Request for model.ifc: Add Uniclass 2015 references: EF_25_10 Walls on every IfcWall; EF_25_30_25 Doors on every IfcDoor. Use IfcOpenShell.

First a look at what the model holds.

```python
import ifcopenshell

model = ifcopenshell.open("model.ifc")
print(model.schema)
print("classifications:", [c.Name for c in model.by_type("IfcClassification")])
for ifc_class in ("IfcDoor", "IfcRoof", "IfcStair", "IfcWall", "IfcWindow"):
    print(ifc_class, len(model.by_type(ifc_class)))
```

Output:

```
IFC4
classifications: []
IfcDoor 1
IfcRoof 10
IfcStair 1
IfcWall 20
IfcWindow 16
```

```python
import ifcopenshell
import ifcopenshell.api.classification

model = ifcopenshell.open("model.ifc")

system = ifcopenshell.api.classification.add_classification(model, classification="Uniclass 2015")

codes = {
    "IfcWall": ("EF_25_10", "Walls"),
    "IfcDoor": ("EF_25_30_25", "Doors"),
}
for ifc_class, (code, name) in codes.items():
    products = model.by_type(ifc_class)
    ifcopenshell.api.classification.add_reference(
        model, products=products, classification=system, identification=code, name=name
    )
    print(code, len(products))

model.write("model-out.ifc")
```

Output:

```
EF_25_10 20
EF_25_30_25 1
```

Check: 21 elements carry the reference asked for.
